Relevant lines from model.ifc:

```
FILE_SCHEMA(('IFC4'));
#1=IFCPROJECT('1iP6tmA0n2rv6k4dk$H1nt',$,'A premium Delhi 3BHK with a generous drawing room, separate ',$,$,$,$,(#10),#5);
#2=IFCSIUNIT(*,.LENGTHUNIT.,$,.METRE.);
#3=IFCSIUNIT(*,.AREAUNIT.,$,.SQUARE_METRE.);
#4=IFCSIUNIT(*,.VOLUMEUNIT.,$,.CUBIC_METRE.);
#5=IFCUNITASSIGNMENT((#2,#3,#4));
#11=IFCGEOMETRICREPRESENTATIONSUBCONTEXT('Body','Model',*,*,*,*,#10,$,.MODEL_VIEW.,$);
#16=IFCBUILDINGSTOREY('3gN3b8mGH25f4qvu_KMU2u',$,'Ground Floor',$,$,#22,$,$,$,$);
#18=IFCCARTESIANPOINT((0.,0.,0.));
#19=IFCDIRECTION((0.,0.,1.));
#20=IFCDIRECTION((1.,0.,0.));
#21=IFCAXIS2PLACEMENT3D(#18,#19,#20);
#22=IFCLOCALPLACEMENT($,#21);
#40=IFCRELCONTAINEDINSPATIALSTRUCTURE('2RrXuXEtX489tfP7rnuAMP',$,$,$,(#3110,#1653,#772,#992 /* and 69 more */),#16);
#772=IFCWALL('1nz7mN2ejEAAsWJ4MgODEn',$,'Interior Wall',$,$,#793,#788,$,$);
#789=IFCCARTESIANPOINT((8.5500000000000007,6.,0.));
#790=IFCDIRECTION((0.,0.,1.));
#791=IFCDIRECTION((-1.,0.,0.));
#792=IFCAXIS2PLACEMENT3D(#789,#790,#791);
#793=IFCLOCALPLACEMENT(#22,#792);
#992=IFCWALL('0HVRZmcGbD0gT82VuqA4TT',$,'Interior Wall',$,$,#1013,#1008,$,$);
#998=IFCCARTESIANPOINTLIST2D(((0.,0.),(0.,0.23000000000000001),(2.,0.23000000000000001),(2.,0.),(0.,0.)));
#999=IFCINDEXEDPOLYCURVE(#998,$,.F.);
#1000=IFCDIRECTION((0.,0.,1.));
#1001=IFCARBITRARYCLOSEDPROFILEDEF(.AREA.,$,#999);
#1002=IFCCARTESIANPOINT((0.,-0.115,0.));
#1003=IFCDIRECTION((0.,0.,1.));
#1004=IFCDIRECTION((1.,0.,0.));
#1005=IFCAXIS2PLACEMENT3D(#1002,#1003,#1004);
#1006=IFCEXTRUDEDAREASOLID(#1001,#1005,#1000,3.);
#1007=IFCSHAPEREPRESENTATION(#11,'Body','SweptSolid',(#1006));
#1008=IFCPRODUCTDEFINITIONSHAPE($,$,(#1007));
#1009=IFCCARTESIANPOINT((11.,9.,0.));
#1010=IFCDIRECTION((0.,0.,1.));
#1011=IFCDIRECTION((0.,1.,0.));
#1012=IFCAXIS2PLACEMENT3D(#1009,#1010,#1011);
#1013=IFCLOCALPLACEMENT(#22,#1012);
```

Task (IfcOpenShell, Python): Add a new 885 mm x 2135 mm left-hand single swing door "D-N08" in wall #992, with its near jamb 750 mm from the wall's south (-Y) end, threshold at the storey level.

```python
import numpy as np
import ifcopenshell
import ifcopenshell.api.feature
import ifcopenshell.api.geometry
import ifcopenshell.api.root
import ifcopenshell.api.spatial
import ifcopenshell.geom
import ifcopenshell.util.element
import ifcopenshell.util.placement
import ifcopenshell.util.representation
import ifcopenshell.util.shape
import ifcopenshell.util.unit

model = ifcopenshell.open("model.ifc")
unit_scale = ifcopenshell.util.unit.calculate_unit_scale(model)
settings = ifcopenshell.geom.settings()


def volume(element):
    """Net volume in cubic metres, openings subtracted."""
    shape = ifcopenshell.geom.create_shape(settings, element)
    return ifcopenshell.util.shape.get_volume(shape.geometry)


wall = model.by_guid("0HVRZmcGbD0gT82VuqA4TT")
storey = ifcopenshell.util.element.get_container(wall, ifc_class="IfcBuildingStorey")
context = ifcopenshell.util.representation.get_context(model, "Model", "Body", "MODEL_VIEW")
before = volume(wall)

width, height, from_end, sill = 0.885, 2.135, 0.75, 0.0  # metres

# The wall runs along its own X axis, and the end named is its -X end.
wall_shape = ifcopenshell.geom.create_shape(settings, wall)
x, y, z = ifcopenshell.util.shape.get_vertices(wall_shape.geometry).T
start = x.min() + from_end
face, thickness = float(y.min()), float(y.max() - y.min())
wall_matrix = ifcopenshell.util.placement.get_local_placement(wall.ObjectPlacement)
level = ifcopenshell.util.placement.get_local_placement(storey.ObjectPlacement)[2, 3]


def in_wall(x, y):
    """Placement at x, y metres in the wall's axes, at sill height."""
    matrix = wall_matrix.copy()
    matrix[:, 3] = wall_matrix @ np.array([x / unit_scale, y / unit_scale, 0.0, 1.0])
    matrix[2, 3] = level + sill / unit_scale
    return matrix


# Opening: a box that overshoots both wall faces by 50 mm.
opening = ifcopenshell.api.root.create_entity(model, ifc_class="IfcOpeningElement", predefined_type="OPENING")
box = ifcopenshell.api.geometry.add_wall_representation(
    model, context=context, length=width, height=height, thickness=thickness + 0.1
)
ifcopenshell.api.geometry.assign_representation(model, product=opening, representation=box)
ifcopenshell.api.geometry.edit_object_placement(model, product=opening, matrix=in_wall(start, face - 0.05), is_si=False)
ifcopenshell.api.feature.add_feature(model, feature=opening, element=wall)

door = ifcopenshell.api.root.create_entity(model, ifc_class="IfcDoor", name="D-N08", predefined_type="DOOR")
door.OverallWidth, door.OverallHeight = width / unit_scale, height / unit_scale
door.OperationType = "SINGLE_SWING_LEFT"
body = ifcopenshell.api.geometry.add_door_representation(
    model,
    context=context,
    overall_width=door.OverallWidth,
    overall_height=door.OverallHeight,
    operation_type="SINGLE_SWING_LEFT",
    lining_properties={"LiningDepth": thickness / unit_scale, "ThresholdDepth": thickness / unit_scale},
)
ifcopenshell.api.geometry.assign_representation(model, product=door, representation=body)
ifcopenshell.api.spatial.assign_container(model, products=[door], relating_structure=storey)
ifcopenshell.api.feature.add_filling(model, opening=opening, element=door)

# The lining spans the wall, so the door starts at the wall face.
ifcopenshell.api.geometry.edit_object_placement(model, product=door, matrix=in_wall(start, face), is_si=False)

after = volume(wall)

print(f"wall volume {before:.3f} -> {after:.3f} m3")

model.write("model_edited.ifc")
```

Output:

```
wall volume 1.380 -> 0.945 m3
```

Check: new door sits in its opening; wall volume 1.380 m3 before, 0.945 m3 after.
